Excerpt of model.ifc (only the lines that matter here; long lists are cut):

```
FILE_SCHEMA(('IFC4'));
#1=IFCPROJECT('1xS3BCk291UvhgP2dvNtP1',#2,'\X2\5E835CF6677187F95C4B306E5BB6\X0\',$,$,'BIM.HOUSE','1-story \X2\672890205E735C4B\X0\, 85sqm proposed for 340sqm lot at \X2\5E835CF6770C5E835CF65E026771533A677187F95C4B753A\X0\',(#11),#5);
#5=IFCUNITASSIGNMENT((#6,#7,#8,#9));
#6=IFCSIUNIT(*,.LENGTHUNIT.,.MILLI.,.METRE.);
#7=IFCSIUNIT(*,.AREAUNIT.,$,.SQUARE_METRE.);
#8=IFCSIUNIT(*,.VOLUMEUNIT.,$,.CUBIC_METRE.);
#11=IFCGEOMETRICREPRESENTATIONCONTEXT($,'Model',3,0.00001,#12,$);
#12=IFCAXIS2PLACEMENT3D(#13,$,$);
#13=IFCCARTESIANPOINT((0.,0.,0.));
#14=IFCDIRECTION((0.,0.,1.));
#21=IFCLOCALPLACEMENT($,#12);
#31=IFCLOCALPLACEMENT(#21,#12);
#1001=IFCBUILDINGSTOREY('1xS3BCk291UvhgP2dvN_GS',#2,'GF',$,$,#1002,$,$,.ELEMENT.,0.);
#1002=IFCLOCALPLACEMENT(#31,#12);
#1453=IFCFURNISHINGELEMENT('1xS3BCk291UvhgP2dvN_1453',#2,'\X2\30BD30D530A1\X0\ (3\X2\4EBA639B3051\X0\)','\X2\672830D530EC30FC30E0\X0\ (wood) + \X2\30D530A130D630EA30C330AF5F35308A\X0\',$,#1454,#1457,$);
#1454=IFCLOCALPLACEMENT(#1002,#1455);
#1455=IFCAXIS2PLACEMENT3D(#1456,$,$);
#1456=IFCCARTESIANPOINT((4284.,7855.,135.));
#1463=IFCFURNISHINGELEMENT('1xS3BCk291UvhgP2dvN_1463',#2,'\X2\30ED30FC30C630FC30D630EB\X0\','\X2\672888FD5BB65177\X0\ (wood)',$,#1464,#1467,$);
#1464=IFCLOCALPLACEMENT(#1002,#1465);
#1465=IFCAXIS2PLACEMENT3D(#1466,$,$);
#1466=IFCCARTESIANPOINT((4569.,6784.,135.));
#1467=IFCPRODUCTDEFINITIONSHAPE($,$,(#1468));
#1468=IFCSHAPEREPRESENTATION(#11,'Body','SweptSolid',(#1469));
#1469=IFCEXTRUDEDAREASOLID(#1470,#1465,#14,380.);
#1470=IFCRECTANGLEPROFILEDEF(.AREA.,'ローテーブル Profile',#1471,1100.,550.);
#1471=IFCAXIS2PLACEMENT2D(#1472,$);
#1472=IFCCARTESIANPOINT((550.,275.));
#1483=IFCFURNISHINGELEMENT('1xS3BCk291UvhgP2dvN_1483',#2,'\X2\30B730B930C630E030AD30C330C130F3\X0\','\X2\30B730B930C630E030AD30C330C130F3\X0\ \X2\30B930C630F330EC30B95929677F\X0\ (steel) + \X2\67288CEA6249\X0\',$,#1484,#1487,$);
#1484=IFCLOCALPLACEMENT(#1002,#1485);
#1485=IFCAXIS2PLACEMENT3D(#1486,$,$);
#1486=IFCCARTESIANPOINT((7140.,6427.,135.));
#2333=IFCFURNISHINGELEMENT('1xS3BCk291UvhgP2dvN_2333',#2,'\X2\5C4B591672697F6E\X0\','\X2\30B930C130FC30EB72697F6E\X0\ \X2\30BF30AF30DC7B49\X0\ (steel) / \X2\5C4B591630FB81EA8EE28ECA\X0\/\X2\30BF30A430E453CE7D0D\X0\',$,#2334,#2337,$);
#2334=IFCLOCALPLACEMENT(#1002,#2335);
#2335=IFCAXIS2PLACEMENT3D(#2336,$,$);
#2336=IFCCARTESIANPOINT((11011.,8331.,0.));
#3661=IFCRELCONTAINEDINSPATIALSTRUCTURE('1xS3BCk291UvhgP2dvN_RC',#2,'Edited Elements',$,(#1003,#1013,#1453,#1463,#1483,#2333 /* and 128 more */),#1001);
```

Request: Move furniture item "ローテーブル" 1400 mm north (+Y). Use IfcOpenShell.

```python
import ifcopenshell
import ifcopenshell.api.geometry
import ifcopenshell.util.placement
import ifcopenshell.util.unit

model = ifcopenshell.open("model.ifc")
unit_scale = ifcopenshell.util.unit.calculate_unit_scale(model)

item = model.by_guid("1xS3BCk291UvhgP2dvN_1463")
matrix = ifcopenshell.util.placement.get_local_placement(item.ObjectPlacement)
matrix[1, 3] += 1.4 / unit_scale
ifcopenshell.api.geometry.edit_object_placement(model, product=item, matrix=matrix, is_si=False)

print(ifcopenshell.util.placement.get_local_placement(item.ObjectPlacement).round(3) + 0.0)

model.write("model_updated.ifc")
```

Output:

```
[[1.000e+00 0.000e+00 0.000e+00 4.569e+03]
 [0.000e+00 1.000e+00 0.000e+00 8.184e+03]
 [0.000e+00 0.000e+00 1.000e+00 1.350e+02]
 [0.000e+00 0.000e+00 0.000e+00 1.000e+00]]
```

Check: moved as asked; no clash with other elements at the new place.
